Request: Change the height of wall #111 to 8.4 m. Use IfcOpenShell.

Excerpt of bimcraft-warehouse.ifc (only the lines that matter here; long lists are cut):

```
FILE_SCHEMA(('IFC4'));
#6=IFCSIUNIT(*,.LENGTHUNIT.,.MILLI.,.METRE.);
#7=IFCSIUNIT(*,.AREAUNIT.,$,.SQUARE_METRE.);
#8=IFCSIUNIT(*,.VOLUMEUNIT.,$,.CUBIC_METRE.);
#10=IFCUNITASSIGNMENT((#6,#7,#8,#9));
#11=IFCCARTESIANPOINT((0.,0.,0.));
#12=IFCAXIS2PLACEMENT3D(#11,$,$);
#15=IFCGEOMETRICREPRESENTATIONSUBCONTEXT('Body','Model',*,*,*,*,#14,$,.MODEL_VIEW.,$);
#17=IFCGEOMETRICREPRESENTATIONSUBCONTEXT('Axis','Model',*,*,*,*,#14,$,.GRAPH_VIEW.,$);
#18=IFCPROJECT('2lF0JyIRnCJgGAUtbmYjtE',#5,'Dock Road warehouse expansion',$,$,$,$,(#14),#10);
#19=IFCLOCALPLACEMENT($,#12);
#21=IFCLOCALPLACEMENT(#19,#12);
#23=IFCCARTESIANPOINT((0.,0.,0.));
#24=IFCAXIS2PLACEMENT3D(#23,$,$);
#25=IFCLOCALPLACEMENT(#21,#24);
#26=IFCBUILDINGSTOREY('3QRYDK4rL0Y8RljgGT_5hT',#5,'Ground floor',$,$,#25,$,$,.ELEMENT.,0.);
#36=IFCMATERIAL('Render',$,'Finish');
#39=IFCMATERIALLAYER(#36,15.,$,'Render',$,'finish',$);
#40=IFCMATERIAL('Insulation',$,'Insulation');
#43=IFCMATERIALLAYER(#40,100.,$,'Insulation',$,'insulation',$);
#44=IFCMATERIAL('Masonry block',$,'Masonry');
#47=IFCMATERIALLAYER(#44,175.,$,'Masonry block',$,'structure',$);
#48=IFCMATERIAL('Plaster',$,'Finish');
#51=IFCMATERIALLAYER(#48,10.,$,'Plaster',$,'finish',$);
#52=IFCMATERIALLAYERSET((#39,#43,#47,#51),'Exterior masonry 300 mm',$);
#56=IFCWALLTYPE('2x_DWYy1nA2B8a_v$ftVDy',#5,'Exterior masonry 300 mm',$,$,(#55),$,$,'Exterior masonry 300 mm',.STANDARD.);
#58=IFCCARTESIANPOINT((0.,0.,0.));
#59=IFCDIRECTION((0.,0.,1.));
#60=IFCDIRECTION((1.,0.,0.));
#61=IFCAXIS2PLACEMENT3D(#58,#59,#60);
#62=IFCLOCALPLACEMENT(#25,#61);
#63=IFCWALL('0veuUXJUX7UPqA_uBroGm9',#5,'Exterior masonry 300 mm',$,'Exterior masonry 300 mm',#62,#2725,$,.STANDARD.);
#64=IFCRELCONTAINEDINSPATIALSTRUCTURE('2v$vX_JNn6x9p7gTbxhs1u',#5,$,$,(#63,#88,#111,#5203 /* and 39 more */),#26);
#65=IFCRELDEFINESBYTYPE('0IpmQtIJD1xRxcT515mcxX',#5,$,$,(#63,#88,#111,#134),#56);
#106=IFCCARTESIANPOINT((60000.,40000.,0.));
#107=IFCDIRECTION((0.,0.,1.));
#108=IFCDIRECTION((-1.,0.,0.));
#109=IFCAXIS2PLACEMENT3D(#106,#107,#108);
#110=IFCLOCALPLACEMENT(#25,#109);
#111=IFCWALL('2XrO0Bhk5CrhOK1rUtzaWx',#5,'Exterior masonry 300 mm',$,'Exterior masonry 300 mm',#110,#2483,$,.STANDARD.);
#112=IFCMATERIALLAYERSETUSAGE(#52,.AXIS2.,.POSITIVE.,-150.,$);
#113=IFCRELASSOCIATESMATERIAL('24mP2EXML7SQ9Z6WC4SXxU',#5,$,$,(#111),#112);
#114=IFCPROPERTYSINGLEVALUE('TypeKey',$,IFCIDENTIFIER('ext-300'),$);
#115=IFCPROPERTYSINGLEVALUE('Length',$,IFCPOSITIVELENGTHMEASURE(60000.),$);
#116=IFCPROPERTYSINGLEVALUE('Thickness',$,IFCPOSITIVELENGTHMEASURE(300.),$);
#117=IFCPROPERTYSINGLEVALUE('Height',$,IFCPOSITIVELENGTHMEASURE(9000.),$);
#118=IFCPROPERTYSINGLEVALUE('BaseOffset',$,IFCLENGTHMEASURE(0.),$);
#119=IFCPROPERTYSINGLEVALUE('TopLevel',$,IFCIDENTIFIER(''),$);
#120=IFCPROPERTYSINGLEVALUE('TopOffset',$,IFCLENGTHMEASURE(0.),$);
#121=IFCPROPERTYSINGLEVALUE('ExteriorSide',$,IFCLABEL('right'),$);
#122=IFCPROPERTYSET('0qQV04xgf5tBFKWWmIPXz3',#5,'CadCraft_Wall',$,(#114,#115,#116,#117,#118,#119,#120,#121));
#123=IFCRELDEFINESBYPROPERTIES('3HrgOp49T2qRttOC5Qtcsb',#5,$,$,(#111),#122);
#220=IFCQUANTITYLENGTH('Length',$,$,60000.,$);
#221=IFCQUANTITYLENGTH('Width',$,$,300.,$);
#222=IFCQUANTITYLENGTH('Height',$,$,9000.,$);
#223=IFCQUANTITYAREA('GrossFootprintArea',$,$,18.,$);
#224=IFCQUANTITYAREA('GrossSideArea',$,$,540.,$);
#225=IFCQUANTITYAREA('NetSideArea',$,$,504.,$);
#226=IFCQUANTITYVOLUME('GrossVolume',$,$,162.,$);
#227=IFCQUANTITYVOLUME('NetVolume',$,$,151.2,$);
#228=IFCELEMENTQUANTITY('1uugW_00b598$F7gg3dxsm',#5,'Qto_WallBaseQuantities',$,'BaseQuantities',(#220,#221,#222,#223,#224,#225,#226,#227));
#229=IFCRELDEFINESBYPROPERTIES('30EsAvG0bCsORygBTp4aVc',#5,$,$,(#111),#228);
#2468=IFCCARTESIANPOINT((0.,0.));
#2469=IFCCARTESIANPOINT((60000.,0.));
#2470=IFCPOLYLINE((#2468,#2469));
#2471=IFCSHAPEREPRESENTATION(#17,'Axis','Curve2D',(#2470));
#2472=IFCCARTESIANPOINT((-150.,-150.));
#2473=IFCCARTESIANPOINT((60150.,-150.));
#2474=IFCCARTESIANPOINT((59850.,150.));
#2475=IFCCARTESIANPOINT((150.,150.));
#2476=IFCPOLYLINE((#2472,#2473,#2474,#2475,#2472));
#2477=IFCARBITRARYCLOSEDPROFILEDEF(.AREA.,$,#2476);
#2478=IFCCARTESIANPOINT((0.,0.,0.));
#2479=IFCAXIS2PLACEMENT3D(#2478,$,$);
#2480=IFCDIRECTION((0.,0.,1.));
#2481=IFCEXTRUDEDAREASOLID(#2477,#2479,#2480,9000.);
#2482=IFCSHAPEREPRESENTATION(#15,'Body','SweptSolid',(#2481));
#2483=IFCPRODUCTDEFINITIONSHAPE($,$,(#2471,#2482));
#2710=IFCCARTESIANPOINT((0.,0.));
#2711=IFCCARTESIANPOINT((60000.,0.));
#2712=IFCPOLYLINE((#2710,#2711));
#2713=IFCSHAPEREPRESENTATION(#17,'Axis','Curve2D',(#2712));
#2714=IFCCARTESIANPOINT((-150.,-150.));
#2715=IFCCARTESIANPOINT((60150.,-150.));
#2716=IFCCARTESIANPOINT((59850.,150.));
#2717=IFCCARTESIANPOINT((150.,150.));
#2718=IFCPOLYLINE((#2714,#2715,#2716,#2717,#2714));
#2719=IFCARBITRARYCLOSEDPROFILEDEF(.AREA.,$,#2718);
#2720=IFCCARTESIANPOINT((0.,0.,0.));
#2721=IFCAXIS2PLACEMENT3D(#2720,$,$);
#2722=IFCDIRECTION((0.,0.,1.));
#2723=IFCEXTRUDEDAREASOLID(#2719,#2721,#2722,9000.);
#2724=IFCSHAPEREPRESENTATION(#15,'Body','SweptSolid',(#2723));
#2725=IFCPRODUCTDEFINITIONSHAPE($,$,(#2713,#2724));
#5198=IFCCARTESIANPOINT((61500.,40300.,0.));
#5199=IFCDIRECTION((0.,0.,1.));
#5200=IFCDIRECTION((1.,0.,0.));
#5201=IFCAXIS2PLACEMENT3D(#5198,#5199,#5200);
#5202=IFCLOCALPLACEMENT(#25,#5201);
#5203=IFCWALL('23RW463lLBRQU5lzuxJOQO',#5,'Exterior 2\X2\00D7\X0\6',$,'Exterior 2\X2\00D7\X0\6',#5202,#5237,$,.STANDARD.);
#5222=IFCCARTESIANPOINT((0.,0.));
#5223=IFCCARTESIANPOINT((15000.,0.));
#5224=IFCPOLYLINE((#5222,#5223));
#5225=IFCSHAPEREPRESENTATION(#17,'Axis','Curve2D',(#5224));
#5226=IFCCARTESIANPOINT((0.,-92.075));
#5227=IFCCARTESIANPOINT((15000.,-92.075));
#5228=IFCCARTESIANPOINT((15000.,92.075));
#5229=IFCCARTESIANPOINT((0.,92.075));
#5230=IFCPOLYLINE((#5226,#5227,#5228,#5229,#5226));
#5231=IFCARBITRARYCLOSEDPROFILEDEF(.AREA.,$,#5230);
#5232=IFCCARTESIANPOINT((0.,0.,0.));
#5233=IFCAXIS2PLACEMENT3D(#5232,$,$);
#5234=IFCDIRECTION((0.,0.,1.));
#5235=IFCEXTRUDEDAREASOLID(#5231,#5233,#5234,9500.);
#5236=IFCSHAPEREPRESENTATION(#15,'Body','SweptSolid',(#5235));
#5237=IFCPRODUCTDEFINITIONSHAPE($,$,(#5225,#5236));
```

```python
import ifcopenshell
import ifcopenshell.api.pset
import ifcopenshell.geom
import ifcopenshell.util.element
import ifcopenshell.util.representation
import ifcopenshell.util.shape
import ifcopenshell.util.unit

model = ifcopenshell.open("bimcraft-warehouse.ifc")
unit_scale = ifcopenshell.util.unit.calculate_unit_scale(model)
area_scale = ifcopenshell.util.unit.calculate_unit_scale(model, "AREAUNIT")
volume_scale = ifcopenshell.util.unit.calculate_unit_scale(model, "VOLUMEUNIT")
settings = ifcopenshell.geom.settings()


def volume(element):
    """Net volume in cubic metres, openings subtracted."""
    shape = ifcopenshell.geom.create_shape(settings, element)
    return ifcopenshell.util.shape.get_volume(shape.geometry)


wall = model.by_guid("2XrO0Bhk5CrhOK1rUtzaWx")
before = volume(wall)

body = ifcopenshell.util.representation.get_representation(wall, "Model", "Body")
solid = body.Items[0]
old_height = solid.Depth
solid.Depth = 8400.0
after = volume(wall)
thickness = 0.3  # wall thickness in metres

# Update the stored height, areas and volumes.
pset = model.by_id(ifcopenshell.util.element.get_pset(wall, "CadCraft_Wall", should_inherit=False)["id"])
ifcopenshell.api.pset.edit_pset(model, pset=pset, properties={
    "Height": model.create_entity("IfcPositiveLengthMeasure", solid.Depth),
})
qto = model.by_id(ifcopenshell.util.element.get_pset(wall, "Qto_WallBaseQuantities", should_inherit=False)["id"])
ifcopenshell.api.pset.edit_qto(model, qto=qto, properties={
    "Height": solid.Depth,
    "GrossSideArea": ifcopenshell.util.element.get_pset(wall, "Qto_WallBaseQuantities", "GrossSideArea") * solid.Depth / old_height,
    "NetSideArea": after / thickness / area_scale,
    "GrossVolume": ifcopenshell.util.element.get_pset(wall, "Qto_WallBaseQuantities", "GrossVolume") * solid.Depth / old_height,
    "NetVolume": after / volume_scale,
})

print(f"height {old_height:g} -> {solid.Depth:g}, volume {before:.3f} -> {after:.3f} m3")

model.write("bimcraft-warehouse_rev.ifc")
```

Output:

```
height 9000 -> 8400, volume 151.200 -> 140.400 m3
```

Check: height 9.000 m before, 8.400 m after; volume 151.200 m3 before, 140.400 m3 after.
